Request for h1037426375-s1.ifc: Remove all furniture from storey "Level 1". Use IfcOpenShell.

First a look at what the model holds.

```python
import ifcopenshell
import ifcopenshell.util.element

model = ifcopenshell.open("h1037426375-s1.ifc")
print(model.schema)
storey = next(s for s in model.by_type("IfcBuildingStorey") if s.Name == "Level 1")
furniture = [e for e in ifcopenshell.util.element.get_decomposition(storey) if e.is_a("IfcFurnishingElement")]
seen = {}
for e in furniture:
    element_type = ifcopenshell.util.element.get_type(e)
    name = element_type.Name if element_type not in (None, e) else None
    seen[name] = seen.get(name, 0) + 1
for name, count in sorted(seen.items(), key=str):
    print(count, "x", name)
```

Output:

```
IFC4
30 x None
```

```python
import ifcopenshell
import ifcopenshell.api.root
import ifcopenshell.util.element

model = ifcopenshell.open("h1037426375-s1.ifc")

storey = next(s for s in model.by_type("IfcBuildingStorey") if s.Name == "Level 1")
furniture = [e for e in ifcopenshell.util.element.get_decomposition(storey) if e.is_a("IfcFurnishingElement")]

for e in furniture:
    ifcopenshell.api.root.remove_product(model, product=e)
print(len(furniture), "removed")

model.write("h1037426375-s1-out.ifc")
```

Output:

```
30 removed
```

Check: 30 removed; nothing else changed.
